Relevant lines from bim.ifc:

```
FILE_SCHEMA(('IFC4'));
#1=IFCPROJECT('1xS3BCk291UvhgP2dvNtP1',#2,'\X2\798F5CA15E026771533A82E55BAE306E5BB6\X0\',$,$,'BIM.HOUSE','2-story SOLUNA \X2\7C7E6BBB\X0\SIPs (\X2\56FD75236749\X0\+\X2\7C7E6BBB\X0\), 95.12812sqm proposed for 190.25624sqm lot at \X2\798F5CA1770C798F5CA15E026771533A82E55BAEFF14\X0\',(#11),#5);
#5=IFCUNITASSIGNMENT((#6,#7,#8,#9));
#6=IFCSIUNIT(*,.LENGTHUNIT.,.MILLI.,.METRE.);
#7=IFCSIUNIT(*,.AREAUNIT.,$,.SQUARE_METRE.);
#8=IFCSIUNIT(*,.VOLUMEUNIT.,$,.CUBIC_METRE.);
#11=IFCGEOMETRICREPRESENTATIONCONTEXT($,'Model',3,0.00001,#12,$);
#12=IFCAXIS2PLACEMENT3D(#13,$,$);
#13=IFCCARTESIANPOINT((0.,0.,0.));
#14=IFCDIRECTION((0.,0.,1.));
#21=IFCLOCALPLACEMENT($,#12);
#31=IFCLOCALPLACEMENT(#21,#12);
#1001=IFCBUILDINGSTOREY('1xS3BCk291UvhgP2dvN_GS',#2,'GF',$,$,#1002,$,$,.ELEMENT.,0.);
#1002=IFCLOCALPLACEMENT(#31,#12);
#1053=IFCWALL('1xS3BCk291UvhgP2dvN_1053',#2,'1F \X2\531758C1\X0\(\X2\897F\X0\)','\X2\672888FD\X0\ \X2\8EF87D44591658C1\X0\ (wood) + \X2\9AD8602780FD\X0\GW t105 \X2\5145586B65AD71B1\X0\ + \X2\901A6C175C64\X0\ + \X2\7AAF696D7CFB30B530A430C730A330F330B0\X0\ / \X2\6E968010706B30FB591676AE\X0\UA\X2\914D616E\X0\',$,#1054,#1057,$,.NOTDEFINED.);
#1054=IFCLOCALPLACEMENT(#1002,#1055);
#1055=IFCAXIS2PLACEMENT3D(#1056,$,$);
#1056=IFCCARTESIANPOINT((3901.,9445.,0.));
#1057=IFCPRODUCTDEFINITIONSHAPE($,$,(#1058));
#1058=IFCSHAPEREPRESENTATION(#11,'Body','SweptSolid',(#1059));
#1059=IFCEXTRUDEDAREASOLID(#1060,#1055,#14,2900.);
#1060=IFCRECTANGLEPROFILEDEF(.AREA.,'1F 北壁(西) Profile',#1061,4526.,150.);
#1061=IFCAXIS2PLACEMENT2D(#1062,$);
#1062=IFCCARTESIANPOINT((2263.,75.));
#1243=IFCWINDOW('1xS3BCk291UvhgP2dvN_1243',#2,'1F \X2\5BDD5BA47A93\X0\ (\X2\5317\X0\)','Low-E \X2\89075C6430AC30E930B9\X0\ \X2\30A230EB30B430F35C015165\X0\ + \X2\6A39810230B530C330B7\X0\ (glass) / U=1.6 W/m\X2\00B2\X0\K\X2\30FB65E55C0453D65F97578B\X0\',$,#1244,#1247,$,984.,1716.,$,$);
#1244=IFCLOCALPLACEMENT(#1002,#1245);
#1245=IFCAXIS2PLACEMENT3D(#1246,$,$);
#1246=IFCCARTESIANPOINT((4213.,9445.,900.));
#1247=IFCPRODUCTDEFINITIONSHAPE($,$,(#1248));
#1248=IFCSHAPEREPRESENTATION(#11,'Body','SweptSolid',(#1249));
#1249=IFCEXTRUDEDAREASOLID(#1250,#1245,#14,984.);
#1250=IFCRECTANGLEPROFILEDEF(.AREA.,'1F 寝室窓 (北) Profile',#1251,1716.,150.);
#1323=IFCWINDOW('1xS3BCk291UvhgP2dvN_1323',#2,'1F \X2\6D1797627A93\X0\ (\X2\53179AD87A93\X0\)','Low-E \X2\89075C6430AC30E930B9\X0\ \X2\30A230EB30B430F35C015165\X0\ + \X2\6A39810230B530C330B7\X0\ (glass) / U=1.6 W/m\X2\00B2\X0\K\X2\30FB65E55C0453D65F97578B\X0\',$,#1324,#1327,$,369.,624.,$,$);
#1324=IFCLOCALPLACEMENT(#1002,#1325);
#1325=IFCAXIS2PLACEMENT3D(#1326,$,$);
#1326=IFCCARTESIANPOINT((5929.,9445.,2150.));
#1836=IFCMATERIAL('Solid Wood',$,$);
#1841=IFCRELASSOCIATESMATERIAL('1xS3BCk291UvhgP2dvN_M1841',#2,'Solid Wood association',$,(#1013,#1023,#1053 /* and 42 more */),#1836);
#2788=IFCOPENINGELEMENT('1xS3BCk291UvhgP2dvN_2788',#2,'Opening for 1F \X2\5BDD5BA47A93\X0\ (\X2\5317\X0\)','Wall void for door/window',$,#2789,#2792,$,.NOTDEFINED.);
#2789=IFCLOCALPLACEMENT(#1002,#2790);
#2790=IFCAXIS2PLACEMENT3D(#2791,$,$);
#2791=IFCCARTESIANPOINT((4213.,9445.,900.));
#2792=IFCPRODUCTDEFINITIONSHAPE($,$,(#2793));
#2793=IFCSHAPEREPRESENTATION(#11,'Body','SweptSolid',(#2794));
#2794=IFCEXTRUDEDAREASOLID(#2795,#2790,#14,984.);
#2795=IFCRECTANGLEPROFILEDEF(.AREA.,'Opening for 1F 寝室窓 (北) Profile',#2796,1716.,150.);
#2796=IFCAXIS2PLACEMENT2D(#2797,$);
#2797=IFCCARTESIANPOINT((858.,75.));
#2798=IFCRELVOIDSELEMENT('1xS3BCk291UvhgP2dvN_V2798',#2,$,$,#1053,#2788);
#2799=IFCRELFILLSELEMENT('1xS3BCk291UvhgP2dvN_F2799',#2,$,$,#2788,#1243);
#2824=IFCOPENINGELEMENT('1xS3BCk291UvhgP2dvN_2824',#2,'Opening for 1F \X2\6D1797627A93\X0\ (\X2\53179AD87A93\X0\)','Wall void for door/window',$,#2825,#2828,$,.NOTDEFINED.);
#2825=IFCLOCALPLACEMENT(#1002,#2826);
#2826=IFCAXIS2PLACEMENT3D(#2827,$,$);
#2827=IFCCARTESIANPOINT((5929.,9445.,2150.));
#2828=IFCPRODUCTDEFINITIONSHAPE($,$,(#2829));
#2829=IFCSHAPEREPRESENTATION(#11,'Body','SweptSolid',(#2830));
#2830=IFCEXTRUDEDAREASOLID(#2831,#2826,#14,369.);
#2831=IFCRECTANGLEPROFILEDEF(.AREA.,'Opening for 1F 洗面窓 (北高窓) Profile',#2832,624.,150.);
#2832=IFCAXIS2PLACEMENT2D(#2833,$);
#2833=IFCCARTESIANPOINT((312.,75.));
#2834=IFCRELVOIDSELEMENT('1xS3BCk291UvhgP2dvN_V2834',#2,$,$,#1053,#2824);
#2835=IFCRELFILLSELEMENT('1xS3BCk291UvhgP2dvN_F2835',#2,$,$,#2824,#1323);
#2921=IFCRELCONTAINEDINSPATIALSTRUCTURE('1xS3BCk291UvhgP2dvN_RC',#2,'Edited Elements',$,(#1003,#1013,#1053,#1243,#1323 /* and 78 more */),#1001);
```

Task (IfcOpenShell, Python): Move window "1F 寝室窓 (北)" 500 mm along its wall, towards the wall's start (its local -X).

```python
import ifcopenshell
import ifcopenshell.api.geometry
import ifcopenshell.util.placement
import ifcopenshell.util.unit

model = ifcopenshell.open("bim.ifc")
unit_scale = ifcopenshell.util.unit.calculate_unit_scale(model)

window = model.by_id(1243)
opening = window.FillsVoids[0].RelatingOpeningElement
wall = opening.VoidsElements[0].RelatingBuildingElement

wall_matrix = ifcopenshell.util.placement.get_local_placement(wall.ObjectPlacement)
shift = wall_matrix[:3, 0] * -0.5 / unit_scale
before = ifcopenshell.util.placement.get_local_placement(window.ObjectPlacement)[:3, 3].copy()

# The window is not placed relative to its opening, so move both.
for product in (opening, window):
    matrix = ifcopenshell.util.placement.get_local_placement(product.ObjectPlacement)
    matrix[:3, 3] += shift
    ifcopenshell.api.geometry.edit_object_placement(model, product=product, matrix=matrix, is_si=False)

after = ifcopenshell.util.placement.get_local_placement(window.ObjectPlacement)[:3, 3]
print("window moved by", (after - before).round(3) + 0.0)

model.write("bim_edited.ifc")
```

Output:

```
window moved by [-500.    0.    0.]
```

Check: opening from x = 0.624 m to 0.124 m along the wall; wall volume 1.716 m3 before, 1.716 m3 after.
